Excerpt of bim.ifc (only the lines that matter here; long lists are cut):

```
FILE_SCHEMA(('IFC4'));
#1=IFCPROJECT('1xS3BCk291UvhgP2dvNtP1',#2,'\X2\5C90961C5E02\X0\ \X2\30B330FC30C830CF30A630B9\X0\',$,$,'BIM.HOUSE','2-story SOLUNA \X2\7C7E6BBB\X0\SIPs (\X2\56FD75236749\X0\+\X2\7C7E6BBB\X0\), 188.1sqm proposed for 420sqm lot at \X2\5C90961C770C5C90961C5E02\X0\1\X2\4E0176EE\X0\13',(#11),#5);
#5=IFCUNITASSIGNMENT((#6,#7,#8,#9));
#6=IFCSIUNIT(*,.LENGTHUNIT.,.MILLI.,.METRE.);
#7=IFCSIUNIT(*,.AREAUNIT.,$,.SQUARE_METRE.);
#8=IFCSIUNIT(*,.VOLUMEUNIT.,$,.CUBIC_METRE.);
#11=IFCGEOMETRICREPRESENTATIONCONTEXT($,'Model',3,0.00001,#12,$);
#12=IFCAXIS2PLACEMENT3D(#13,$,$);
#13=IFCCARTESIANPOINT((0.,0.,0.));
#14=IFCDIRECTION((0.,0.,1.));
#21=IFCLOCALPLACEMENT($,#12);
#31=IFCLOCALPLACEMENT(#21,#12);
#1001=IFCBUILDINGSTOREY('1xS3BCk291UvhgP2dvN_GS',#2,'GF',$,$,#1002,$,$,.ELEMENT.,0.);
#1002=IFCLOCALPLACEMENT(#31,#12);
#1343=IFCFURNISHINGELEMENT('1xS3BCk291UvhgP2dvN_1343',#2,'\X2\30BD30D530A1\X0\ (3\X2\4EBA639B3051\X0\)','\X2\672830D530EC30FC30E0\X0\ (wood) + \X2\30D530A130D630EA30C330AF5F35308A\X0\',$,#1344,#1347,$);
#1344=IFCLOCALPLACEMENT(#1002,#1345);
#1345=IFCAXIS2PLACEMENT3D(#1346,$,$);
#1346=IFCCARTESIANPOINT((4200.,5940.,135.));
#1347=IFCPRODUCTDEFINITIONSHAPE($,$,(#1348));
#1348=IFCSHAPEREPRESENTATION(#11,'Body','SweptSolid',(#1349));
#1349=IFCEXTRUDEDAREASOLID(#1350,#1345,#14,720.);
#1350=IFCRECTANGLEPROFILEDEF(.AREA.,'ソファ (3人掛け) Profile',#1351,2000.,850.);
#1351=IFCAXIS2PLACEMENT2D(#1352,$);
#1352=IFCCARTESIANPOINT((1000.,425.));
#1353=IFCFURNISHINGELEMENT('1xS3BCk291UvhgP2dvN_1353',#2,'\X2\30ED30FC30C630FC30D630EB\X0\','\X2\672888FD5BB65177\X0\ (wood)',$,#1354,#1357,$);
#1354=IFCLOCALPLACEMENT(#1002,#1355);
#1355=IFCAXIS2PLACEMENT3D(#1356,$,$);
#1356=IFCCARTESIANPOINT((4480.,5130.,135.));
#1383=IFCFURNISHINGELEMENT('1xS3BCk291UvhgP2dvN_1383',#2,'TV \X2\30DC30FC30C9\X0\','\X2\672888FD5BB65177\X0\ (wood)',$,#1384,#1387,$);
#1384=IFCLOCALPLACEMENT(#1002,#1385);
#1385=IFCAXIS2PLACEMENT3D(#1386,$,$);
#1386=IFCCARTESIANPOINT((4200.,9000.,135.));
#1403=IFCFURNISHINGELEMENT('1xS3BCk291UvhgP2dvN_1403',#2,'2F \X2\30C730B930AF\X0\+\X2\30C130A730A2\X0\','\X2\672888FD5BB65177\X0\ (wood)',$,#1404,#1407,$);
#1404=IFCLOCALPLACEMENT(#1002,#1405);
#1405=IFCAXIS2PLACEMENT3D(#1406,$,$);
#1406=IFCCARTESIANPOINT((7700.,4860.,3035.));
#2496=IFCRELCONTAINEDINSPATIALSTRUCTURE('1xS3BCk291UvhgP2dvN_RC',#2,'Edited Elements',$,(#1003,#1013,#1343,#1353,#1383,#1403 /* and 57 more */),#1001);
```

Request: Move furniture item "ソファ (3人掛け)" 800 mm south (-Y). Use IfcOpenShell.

```python
import ifcopenshell
import ifcopenshell.api.geometry
import ifcopenshell.util.placement
import ifcopenshell.util.unit

model = ifcopenshell.open("bim.ifc")
unit_scale = ifcopenshell.util.unit.calculate_unit_scale(model)

item = model.by_guid("1xS3BCk291UvhgP2dvN_1343")
matrix = ifcopenshell.util.placement.get_local_placement(item.ObjectPlacement)
matrix[1, 3] -= 0.8 / unit_scale
ifcopenshell.api.geometry.edit_object_placement(model, product=item, matrix=matrix, is_si=False)

print(ifcopenshell.util.placement.get_local_placement(item.ObjectPlacement).round(3) + 0.0)

model.write("bim_rev.ifc")
```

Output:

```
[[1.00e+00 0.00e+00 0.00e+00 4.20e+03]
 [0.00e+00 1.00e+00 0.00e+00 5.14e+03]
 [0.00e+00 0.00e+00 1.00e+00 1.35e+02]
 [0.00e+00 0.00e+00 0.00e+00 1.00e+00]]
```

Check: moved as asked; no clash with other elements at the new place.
